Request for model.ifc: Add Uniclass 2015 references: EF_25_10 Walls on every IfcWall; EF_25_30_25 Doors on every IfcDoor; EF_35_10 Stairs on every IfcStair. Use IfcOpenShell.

First a look at what the model holds.

```python
import ifcopenshell

model = ifcopenshell.open("model.ifc")
print(model.schema)
print("classifications:", [c.Name for c in model.by_type("IfcClassification")])
for ifc_class in ("IfcDoor", "IfcRoof", "IfcStair", "IfcWall", "IfcWindow"):
    print(ifc_class, len(model.by_type(ifc_class)))
```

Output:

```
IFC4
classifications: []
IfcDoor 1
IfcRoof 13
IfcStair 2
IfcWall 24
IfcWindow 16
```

```python
import ifcopenshell
import ifcopenshell.api.classification

model = ifcopenshell.open("model.ifc")

system = ifcopenshell.api.classification.add_classification(model, classification="Uniclass 2015")

codes = {
    "IfcWall": ("EF_25_10", "Walls"),
    "IfcDoor": ("EF_25_30_25", "Doors"),
    "IfcStair": ("EF_35_10", "Stairs"),
}
for ifc_class, (code, name) in codes.items():
    products = model.by_type(ifc_class)
    ifcopenshell.api.classification.add_reference(
        model, products=products, classification=system, identification=code, name=name
    )
    print(code, len(products))

model.write("model-out.ifc")
```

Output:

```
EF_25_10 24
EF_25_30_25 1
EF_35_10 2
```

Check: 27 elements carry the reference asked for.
